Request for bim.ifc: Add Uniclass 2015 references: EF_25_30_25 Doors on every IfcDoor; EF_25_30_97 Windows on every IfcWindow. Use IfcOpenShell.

First a look at what the model holds.

```python
import ifcopenshell

model = ifcopenshell.open("bim.ifc")
print(model.schema)
print("classifications:", [c.Name for c in model.by_type("IfcClassification")])
for ifc_class in ("IfcDoor", "IfcRoof", "IfcStair", "IfcWall", "IfcWindow"):
    print(ifc_class, len(model.by_type(ifc_class)))
```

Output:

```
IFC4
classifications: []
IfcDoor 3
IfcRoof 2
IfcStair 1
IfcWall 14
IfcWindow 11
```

```python
import ifcopenshell
import ifcopenshell.api.classification

model = ifcopenshell.open("bim.ifc")

system = ifcopenshell.api.classification.add_classification(model, classification="Uniclass 2015")

codes = {
    "IfcDoor": ("EF_25_30_25", "Doors"),
    "IfcWindow": ("EF_25_30_97", "Windows"),
}
for ifc_class, (code, name) in codes.items():
    products = model.by_type(ifc_class)
    ifcopenshell.api.classification.add_reference(
        model, products=products, classification=system, identification=code, name=name
    )
    print(code, len(products))

model.write("bim_edited.ifc")
```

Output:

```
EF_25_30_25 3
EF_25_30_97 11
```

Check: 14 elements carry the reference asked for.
